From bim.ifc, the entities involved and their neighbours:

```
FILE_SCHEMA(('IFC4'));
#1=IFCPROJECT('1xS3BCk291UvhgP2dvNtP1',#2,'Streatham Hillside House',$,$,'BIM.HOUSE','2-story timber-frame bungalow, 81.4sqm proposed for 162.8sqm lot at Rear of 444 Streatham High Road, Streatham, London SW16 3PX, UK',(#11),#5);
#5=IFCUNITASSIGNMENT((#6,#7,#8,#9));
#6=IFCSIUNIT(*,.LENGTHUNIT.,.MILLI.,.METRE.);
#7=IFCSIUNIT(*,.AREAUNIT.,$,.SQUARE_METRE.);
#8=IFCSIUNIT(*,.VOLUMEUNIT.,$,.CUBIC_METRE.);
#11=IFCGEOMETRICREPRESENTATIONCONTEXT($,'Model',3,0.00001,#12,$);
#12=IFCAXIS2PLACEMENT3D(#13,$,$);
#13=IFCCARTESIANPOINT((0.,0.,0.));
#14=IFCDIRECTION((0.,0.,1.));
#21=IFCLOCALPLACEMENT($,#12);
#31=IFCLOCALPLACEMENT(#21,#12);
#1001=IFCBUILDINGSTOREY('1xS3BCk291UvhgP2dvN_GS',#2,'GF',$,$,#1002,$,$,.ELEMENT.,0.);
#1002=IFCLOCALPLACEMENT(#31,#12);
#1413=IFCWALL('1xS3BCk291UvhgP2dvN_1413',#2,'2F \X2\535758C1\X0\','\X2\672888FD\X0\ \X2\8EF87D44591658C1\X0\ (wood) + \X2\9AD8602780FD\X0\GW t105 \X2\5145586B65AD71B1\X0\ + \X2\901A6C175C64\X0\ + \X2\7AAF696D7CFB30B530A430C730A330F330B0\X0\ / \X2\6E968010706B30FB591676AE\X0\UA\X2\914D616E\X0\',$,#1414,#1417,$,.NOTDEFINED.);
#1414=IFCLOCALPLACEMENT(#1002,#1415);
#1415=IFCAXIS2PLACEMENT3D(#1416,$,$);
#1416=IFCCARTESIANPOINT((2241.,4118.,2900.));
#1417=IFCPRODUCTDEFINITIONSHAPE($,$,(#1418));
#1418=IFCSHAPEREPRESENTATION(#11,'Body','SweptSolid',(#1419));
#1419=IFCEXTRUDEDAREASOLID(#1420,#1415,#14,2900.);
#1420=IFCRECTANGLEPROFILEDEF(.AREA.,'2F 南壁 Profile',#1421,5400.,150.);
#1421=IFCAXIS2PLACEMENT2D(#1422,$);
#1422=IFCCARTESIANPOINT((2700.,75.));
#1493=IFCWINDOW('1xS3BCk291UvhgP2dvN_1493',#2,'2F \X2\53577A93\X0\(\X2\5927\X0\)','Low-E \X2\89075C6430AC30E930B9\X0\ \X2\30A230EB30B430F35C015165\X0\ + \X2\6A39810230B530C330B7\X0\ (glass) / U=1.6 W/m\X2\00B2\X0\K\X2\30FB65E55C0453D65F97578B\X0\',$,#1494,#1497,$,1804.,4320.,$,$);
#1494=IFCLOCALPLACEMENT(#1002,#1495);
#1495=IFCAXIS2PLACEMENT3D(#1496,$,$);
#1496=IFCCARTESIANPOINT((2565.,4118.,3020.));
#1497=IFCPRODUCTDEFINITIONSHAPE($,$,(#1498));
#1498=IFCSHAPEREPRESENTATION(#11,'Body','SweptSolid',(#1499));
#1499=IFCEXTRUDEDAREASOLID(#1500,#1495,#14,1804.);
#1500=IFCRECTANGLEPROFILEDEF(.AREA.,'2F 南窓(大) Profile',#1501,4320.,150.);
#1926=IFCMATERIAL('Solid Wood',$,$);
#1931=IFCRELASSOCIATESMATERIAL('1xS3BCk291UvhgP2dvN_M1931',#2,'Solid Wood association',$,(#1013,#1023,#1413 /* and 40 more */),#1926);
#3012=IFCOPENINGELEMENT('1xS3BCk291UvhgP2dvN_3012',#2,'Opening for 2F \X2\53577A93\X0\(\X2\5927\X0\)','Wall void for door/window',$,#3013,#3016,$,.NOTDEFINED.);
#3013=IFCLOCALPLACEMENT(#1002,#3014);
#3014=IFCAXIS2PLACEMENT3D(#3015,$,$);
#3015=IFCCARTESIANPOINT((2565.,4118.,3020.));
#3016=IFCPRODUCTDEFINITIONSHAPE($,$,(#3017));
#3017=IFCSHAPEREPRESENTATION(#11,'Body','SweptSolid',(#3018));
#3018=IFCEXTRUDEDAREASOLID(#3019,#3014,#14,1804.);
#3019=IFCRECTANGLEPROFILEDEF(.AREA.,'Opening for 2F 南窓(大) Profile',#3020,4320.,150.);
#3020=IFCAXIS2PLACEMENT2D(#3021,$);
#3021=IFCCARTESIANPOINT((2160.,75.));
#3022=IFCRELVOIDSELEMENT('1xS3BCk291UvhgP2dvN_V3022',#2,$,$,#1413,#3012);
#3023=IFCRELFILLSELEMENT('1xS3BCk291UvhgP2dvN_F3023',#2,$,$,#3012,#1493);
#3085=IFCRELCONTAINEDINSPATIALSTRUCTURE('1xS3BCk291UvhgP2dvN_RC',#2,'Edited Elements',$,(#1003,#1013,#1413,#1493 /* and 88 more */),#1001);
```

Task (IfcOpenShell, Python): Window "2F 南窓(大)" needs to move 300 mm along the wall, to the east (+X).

```python
import ifcopenshell
import ifcopenshell.api.geometry
import ifcopenshell.util.placement
import ifcopenshell.util.unit

model = ifcopenshell.open("bim.ifc")
unit_scale = ifcopenshell.util.unit.calculate_unit_scale(model)

window = model.by_guid("1xS3BCk291UvhgP2dvN_1493")
opening = window.FillsVoids[0].RelatingOpeningElement
wall = opening.VoidsElements[0].RelatingBuildingElement

wall_matrix = ifcopenshell.util.placement.get_local_placement(wall.ObjectPlacement)
shift = wall_matrix[:3, 0] * 0.3 / unit_scale
before = ifcopenshell.util.placement.get_local_placement(window.ObjectPlacement)[:3, 3].copy()

# The window is not placed relative to its opening, so move both.
for product in (opening, window):
    matrix = ifcopenshell.util.placement.get_local_placement(product.ObjectPlacement)
    matrix[:3, 3] += shift
    ifcopenshell.api.geometry.edit_object_placement(model, product=product, matrix=matrix, is_si=False)

after = ifcopenshell.util.placement.get_local_placement(window.ObjectPlacement)[:3, 3]
print("window moved by", (after - before).round(3) + 0.0)

model.write("bim_rev.ifc")
```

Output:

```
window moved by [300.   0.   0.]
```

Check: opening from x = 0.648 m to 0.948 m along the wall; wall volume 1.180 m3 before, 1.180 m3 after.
